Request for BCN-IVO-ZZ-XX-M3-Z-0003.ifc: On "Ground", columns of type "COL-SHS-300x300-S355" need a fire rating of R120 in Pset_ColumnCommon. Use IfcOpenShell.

First a look at what the model holds.

```python
import ifcopenshell
import ifcopenshell.util.element

model = ifcopenshell.open("BCN-IVO-ZZ-XX-M3-Z-0003.ifc")
print(model.schema)
storey = next(s for s in model.by_type("IfcBuildingStorey") if s.Name == "Ground")
columns = [e for e in ifcopenshell.util.element.get_decomposition(storey) if e.is_a("IfcColumn")]
seen = {}
for e in columns:
    element_type = ifcopenshell.util.element.get_type(e)
    key = (element_type.Name if element_type != e and element_type else None, ifcopenshell.util.element.get_pset(e, "Pset_ColumnCommon", "FireRating"))
    seen[key] = seen.get(key, 0) + 1
for (name, value), count in sorted(seen.items(), key=str):
    print(count, "x", name, "|", value)
```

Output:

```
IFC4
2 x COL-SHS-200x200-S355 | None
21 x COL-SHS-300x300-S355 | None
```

```python
import ifcopenshell
import ifcopenshell.api.pset
import ifcopenshell.util.element

model = ifcopenshell.open("BCN-IVO-ZZ-XX-M3-Z-0003.ifc")

storey = next(s for s in model.by_type("IfcBuildingStorey") if s.Name == "Ground")
columns = [e for e in ifcopenshell.util.element.get_decomposition(storey) if e.is_a("IfcColumn")]

count = 0
for e in columns:
    element_type = ifcopenshell.util.element.get_type(e)
    if element_type in (None, e) or element_type.Name != "COL-SHS-300x300-S355":
        continue
    # add_pset returns the element's existing set when there is one.
    pset = ifcopenshell.api.pset.add_pset(model, product=e, name="Pset_ColumnCommon")
    ifcopenshell.api.pset.edit_pset(model, pset=pset, properties={"FireRating": "R120"})
    count += 1

print(count, "columns updated")

model.write("BCN-IVO-ZZ-XX-M3-Z-0003_rev.ifc")
```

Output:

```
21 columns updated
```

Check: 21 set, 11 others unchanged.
